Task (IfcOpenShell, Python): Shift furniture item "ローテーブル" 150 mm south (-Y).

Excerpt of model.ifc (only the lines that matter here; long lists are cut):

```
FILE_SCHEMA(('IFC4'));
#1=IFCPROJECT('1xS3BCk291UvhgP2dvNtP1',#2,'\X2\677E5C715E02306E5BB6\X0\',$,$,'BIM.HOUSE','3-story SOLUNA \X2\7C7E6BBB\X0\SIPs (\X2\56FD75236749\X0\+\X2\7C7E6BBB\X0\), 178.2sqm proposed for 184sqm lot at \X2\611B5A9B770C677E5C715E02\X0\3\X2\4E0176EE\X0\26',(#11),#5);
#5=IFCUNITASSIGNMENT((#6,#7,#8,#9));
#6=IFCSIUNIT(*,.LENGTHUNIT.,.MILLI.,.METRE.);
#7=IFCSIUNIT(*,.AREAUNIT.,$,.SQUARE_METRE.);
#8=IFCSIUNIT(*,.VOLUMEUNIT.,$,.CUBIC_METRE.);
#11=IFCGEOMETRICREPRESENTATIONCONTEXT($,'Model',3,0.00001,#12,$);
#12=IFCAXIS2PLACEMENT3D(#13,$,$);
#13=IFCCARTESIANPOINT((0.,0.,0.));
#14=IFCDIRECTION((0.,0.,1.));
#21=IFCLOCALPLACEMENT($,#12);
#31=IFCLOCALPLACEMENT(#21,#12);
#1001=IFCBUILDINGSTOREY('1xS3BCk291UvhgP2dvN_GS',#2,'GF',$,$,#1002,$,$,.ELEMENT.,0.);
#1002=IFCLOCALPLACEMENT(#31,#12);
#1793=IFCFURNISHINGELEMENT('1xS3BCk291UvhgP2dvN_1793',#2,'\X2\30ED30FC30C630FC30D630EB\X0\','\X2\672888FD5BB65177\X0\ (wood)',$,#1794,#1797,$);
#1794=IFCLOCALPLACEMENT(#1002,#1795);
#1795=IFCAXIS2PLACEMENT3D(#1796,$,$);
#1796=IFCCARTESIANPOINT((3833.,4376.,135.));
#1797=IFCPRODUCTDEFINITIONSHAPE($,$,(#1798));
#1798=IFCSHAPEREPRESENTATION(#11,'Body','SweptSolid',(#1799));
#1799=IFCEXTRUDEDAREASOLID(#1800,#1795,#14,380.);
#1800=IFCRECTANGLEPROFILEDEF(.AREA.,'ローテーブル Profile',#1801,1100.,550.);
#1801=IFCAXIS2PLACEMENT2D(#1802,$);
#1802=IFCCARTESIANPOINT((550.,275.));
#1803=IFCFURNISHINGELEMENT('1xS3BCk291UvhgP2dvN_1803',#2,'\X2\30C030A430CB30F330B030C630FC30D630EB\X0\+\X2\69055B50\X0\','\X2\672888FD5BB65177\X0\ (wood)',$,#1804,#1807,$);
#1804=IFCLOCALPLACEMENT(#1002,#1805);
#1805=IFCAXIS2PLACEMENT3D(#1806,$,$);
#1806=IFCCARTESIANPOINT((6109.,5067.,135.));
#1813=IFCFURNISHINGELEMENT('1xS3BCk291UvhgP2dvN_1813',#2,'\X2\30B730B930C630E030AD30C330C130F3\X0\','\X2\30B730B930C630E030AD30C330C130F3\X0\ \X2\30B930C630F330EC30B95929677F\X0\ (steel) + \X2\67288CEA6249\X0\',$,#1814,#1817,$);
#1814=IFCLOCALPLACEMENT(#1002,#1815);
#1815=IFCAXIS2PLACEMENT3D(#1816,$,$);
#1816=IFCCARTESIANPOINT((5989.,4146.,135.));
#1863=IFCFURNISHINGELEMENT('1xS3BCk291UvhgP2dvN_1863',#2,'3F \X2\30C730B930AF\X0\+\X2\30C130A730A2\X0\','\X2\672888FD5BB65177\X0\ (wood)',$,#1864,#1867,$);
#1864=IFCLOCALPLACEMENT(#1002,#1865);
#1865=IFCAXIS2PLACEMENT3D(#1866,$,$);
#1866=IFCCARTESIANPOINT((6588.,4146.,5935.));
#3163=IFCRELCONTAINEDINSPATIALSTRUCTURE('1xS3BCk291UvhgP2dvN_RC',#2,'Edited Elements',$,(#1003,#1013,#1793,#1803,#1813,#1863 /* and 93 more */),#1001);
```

```python
import ifcopenshell
import ifcopenshell.api.geometry
import ifcopenshell.util.placement
import ifcopenshell.util.unit

model = ifcopenshell.open("model.ifc")
unit_scale = ifcopenshell.util.unit.calculate_unit_scale(model)

item = model.by_guid("1xS3BCk291UvhgP2dvN_1793")
matrix = ifcopenshell.util.placement.get_local_placement(item.ObjectPlacement)
matrix[1, 3] -= 0.15 / unit_scale
ifcopenshell.api.geometry.edit_object_placement(model, product=item, matrix=matrix, is_si=False)

print(ifcopenshell.util.placement.get_local_placement(item.ObjectPlacement).round(3) + 0.0)

model.write("model_edited.ifc")
```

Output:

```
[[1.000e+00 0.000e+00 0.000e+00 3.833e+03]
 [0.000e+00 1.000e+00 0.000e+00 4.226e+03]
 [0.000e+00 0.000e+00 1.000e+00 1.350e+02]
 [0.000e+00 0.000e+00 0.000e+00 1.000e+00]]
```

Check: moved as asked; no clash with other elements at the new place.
